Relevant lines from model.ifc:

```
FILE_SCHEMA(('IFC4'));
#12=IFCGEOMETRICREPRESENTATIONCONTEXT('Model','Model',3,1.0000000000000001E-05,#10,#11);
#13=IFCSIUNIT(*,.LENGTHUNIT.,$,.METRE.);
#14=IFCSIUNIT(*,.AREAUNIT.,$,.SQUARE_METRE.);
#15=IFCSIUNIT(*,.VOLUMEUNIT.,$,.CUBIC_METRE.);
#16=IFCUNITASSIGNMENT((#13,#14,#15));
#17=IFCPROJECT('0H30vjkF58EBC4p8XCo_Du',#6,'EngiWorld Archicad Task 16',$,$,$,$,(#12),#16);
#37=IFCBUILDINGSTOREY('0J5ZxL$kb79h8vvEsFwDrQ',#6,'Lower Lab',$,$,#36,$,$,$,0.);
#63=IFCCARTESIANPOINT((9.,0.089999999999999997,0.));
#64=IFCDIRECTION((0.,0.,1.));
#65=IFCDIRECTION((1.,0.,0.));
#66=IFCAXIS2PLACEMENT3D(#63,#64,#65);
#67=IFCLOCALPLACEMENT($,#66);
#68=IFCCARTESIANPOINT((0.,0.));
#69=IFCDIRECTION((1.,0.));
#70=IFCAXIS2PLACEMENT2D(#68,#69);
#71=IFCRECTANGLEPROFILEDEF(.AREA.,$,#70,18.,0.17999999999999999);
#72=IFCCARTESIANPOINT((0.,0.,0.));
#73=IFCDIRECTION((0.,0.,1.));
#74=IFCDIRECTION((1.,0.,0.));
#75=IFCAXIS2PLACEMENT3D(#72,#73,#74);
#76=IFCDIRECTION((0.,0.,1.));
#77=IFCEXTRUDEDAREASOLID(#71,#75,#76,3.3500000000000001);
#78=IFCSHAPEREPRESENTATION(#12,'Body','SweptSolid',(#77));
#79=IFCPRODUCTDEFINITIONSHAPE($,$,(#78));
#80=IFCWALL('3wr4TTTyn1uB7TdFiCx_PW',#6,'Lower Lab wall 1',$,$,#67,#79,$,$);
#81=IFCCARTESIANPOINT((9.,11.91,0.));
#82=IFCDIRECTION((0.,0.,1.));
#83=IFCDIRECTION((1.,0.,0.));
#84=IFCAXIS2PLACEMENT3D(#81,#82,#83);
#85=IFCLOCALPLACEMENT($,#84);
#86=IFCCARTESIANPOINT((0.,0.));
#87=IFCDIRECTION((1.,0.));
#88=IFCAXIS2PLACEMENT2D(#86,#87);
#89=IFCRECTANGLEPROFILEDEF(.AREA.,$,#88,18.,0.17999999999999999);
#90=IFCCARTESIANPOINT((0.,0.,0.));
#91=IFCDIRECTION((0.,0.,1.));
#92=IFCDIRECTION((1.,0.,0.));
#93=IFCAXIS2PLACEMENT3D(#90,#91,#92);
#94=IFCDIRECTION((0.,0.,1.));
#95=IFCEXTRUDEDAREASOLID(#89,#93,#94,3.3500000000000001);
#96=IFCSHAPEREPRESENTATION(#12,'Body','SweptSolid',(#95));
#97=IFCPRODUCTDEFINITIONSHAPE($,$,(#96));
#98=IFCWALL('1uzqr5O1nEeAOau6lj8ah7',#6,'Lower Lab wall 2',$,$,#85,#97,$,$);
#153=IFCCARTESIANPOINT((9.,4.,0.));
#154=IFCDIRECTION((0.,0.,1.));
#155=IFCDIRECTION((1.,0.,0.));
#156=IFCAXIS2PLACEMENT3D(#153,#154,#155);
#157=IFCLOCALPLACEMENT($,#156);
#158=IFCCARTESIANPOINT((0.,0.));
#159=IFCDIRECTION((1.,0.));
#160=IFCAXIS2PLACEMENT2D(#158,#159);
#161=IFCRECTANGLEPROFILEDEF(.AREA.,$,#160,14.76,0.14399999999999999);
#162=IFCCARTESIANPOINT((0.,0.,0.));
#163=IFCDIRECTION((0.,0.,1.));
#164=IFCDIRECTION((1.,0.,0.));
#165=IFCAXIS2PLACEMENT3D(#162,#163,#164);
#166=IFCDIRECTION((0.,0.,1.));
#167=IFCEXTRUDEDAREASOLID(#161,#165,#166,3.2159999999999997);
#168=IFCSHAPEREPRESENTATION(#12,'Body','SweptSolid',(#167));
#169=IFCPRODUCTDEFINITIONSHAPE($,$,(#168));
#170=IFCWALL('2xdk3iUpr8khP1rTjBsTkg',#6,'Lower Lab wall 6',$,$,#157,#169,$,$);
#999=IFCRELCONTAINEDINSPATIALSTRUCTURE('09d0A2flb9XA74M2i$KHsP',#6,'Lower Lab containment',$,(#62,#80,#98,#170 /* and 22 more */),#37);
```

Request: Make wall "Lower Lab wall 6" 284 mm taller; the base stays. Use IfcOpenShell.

```python
import ifcopenshell
import ifcopenshell.geom
import ifcopenshell.util.shape

model = ifcopenshell.open("model.ifc")
settings = ifcopenshell.geom.settings()


def volume(element):
    """Net volume in cubic metres, openings subtracted."""
    shape = ifcopenshell.geom.create_shape(settings, element)
    return ifcopenshell.util.shape.get_volume(shape.geometry)


wall = model.by_guid("2xdk3iUpr8khP1rTjBsTkg")
before = volume(wall)

body = next(r for r in wall.Representation.Representations if r.RepresentationIdentifier == "Body")
solid = body.Items[0]
old_height = solid.Depth
solid.Depth += 0.284
after = volume(wall)

print(f"height {old_height:g} -> {solid.Depth:g}, volume {before:.3f} -> {after:.3f} m3")

model.write("model-out.ifc")
```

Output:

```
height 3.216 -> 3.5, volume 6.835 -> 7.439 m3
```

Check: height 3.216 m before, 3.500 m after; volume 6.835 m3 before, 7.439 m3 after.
